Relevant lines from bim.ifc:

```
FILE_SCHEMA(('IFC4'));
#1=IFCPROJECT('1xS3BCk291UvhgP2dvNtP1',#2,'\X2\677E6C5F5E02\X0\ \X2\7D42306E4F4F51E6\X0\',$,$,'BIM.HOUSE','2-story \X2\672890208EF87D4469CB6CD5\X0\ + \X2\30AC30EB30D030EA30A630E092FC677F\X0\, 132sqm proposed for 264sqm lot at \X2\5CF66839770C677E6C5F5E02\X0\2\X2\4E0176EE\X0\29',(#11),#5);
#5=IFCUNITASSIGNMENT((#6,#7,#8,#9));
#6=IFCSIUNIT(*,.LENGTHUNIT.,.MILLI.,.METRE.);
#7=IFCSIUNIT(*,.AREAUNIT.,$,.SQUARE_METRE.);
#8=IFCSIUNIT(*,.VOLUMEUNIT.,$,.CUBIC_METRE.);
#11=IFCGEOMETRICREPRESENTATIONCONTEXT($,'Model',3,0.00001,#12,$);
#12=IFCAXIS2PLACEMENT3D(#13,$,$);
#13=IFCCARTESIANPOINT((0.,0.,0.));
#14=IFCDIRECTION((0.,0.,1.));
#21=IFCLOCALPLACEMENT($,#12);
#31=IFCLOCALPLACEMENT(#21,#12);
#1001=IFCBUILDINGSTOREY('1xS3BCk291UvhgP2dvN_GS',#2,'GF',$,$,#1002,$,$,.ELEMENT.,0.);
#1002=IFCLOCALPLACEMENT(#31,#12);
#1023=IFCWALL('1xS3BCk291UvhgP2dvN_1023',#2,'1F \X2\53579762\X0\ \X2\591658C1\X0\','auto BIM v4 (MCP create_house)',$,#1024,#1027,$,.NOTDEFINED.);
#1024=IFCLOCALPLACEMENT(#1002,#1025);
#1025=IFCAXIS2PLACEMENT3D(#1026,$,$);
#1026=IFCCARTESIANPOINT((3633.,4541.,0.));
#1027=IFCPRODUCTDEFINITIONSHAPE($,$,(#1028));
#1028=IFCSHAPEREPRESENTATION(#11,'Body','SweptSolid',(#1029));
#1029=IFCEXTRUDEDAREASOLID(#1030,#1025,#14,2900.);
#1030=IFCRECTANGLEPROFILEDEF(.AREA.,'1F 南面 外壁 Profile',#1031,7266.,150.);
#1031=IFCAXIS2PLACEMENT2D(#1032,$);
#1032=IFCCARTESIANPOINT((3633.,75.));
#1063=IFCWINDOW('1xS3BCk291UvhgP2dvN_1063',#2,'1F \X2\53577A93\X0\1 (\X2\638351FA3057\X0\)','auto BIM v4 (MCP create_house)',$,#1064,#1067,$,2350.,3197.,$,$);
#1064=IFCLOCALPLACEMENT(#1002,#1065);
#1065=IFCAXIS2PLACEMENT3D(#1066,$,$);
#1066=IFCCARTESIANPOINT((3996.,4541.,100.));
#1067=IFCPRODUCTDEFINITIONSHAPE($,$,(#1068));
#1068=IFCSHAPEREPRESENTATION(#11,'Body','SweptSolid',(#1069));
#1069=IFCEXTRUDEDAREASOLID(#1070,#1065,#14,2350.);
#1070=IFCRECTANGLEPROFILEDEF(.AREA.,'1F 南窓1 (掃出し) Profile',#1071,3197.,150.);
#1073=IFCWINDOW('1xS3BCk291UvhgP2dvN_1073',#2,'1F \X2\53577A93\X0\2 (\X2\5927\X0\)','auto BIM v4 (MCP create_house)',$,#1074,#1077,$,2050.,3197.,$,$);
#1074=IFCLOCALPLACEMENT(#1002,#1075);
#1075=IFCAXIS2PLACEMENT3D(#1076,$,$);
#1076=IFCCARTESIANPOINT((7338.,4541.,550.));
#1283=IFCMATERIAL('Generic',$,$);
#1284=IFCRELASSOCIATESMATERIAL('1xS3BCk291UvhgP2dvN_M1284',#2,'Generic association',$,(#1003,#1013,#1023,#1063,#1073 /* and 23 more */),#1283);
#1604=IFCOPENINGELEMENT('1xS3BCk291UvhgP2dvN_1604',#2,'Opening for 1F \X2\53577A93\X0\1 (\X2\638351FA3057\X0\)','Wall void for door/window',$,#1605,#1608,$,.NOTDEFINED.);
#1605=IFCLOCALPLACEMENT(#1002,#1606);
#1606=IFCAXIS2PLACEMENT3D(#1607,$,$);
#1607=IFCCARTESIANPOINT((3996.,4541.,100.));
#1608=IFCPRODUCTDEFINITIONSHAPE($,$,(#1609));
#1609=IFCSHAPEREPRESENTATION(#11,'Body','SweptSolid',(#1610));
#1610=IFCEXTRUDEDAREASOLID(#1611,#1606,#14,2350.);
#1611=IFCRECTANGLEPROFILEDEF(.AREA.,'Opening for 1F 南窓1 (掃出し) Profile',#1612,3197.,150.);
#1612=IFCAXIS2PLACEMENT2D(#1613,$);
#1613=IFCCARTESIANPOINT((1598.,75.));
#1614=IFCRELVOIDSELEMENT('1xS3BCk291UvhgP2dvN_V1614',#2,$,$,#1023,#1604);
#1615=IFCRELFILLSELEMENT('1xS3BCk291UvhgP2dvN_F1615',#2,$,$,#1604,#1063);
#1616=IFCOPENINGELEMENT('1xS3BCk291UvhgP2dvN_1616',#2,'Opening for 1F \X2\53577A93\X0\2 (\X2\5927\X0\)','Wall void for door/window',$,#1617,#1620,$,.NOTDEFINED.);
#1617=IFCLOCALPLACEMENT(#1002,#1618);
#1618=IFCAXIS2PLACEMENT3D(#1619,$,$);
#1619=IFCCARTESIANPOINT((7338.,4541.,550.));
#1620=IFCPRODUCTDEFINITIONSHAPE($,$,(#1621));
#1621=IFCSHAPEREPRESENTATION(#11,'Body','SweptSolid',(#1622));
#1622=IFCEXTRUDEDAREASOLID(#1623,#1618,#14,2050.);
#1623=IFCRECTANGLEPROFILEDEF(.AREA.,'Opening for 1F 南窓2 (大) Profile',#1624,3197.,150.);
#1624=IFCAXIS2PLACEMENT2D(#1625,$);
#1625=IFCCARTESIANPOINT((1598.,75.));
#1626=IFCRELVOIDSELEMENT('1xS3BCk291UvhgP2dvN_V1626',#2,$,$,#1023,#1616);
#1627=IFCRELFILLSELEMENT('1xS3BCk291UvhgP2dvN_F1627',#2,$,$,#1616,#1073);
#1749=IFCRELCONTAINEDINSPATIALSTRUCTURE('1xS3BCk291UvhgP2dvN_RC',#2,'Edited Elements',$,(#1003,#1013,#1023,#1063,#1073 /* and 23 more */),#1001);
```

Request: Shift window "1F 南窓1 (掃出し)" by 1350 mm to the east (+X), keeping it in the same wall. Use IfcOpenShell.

```python
import ifcopenshell
import ifcopenshell.api.geometry
import ifcopenshell.util.placement
import ifcopenshell.util.unit

model = ifcopenshell.open("bim.ifc")
unit_scale = ifcopenshell.util.unit.calculate_unit_scale(model)

window = model.by_guid("1xS3BCk291UvhgP2dvN_1063")
opening = window.FillsVoids[0].RelatingOpeningElement
wall = opening.VoidsElements[0].RelatingBuildingElement

wall_matrix = ifcopenshell.util.placement.get_local_placement(wall.ObjectPlacement)
shift = wall_matrix[:3, 0] * 1.35 / unit_scale
before = ifcopenshell.util.placement.get_local_placement(window.ObjectPlacement)[:3, 3].copy()

# The window is not placed relative to its opening, so move both.
for product in (opening, window):
    matrix = ifcopenshell.util.placement.get_local_placement(product.ObjectPlacement)
    matrix[:3, 3] += shift
    ifcopenshell.api.geometry.edit_object_placement(model, product=product, matrix=matrix, is_si=False)

after = ifcopenshell.util.placement.get_local_placement(window.ObjectPlacement)[:3, 3]
print("window moved by", (after - before).round(3) + 0.0)

model.write("bim_updated.ifc")
```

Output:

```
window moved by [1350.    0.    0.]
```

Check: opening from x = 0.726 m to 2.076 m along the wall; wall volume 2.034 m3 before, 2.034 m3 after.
